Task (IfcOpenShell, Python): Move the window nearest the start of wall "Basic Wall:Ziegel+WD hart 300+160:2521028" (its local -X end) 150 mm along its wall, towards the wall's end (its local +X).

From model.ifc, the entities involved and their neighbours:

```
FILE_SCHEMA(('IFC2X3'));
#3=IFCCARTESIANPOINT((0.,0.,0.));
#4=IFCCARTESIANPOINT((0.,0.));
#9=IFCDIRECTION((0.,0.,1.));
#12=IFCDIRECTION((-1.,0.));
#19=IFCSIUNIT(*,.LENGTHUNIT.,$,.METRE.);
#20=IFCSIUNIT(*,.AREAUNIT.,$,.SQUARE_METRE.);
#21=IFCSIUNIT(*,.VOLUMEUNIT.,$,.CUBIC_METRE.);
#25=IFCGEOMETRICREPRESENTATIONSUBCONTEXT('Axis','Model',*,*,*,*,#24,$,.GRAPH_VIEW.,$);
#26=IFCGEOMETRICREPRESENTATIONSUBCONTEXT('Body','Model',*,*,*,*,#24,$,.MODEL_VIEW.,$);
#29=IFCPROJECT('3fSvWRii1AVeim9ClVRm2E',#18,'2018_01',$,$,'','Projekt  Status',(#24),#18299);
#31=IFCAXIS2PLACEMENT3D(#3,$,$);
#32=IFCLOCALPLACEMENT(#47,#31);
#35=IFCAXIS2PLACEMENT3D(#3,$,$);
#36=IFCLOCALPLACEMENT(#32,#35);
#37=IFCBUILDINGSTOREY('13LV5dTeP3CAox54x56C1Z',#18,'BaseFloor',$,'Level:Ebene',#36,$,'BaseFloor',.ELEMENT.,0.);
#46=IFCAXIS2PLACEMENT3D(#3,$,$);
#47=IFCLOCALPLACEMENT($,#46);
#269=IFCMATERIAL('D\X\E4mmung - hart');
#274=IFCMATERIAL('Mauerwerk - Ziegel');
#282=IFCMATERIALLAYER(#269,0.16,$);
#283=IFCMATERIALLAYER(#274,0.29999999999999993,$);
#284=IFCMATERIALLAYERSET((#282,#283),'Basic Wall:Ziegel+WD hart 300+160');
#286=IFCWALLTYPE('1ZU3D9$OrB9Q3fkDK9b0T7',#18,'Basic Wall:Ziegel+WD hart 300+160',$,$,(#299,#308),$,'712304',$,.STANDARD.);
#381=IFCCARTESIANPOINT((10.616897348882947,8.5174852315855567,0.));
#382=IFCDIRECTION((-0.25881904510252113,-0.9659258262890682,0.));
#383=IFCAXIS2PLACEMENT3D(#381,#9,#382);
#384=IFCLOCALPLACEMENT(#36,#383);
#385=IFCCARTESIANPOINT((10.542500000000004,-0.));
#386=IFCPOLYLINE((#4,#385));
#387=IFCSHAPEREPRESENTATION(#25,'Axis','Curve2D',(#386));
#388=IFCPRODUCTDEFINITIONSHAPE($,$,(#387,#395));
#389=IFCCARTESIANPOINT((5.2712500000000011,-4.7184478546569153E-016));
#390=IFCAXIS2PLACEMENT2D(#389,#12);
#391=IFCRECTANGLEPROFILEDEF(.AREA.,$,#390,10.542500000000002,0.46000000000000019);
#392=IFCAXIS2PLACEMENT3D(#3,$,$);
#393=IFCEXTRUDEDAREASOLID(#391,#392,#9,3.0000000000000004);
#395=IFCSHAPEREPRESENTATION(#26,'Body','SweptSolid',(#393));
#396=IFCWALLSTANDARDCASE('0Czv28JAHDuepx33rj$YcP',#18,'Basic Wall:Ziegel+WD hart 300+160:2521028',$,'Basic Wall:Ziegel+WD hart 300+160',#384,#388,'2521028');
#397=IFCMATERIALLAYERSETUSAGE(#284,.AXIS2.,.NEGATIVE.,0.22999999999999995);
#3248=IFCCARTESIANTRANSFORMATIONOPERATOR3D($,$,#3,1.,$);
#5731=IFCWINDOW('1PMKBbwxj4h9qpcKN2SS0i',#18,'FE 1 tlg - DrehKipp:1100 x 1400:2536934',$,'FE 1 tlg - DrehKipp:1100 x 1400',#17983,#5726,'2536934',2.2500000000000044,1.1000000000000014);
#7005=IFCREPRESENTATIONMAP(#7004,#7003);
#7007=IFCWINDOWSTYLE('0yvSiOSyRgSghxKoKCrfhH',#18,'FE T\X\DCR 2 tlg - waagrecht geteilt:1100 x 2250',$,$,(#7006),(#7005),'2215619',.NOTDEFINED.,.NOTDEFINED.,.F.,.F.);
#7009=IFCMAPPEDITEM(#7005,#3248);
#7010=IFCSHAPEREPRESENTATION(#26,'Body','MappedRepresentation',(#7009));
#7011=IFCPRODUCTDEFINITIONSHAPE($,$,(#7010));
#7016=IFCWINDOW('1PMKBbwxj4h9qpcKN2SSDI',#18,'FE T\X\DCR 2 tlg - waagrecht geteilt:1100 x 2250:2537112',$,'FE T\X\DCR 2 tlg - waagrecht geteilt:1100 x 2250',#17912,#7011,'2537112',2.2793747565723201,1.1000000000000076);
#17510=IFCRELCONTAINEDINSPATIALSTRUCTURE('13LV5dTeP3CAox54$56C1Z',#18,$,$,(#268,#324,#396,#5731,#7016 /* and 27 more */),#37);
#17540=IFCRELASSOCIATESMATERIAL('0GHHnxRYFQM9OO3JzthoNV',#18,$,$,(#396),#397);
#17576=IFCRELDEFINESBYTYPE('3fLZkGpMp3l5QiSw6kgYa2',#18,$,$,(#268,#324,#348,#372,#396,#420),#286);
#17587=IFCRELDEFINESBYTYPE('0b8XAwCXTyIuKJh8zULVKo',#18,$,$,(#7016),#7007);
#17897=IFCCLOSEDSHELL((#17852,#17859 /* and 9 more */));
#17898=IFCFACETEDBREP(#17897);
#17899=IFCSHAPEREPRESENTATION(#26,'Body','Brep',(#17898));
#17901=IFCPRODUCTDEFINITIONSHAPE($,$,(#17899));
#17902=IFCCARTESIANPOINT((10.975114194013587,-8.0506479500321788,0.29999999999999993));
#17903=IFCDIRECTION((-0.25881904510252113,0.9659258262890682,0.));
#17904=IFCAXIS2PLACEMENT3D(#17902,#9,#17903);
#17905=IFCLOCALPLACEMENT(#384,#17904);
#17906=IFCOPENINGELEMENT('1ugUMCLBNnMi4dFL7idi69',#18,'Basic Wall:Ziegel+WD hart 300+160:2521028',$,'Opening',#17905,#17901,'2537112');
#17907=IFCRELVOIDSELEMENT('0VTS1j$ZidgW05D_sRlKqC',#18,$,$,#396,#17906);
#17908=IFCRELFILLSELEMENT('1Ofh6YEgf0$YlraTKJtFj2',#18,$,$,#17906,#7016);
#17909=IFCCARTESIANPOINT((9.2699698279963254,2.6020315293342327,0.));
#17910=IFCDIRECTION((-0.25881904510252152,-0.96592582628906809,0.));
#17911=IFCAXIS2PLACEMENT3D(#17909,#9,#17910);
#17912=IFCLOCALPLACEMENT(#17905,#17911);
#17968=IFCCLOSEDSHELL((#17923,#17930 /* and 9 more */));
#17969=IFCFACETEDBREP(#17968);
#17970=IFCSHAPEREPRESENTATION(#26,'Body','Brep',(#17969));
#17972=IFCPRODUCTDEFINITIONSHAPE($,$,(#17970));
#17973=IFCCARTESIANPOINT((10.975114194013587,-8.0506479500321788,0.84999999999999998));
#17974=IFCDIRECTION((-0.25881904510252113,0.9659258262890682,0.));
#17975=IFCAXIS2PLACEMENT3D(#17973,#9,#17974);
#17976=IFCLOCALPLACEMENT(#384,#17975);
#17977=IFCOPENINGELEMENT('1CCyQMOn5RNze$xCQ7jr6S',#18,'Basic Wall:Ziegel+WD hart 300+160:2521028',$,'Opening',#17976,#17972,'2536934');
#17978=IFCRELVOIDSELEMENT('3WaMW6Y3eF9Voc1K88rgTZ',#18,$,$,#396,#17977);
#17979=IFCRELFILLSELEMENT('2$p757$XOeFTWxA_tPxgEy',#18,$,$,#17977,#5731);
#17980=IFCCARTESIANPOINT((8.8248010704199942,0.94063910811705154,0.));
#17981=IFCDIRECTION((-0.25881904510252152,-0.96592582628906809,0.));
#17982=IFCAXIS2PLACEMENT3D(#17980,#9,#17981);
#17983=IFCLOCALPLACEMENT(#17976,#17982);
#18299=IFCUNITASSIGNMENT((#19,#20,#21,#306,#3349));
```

```python
import ifcopenshell
import ifcopenshell.api.geometry
import ifcopenshell.util.placement
import ifcopenshell.util.unit

model = ifcopenshell.open("model.ifc")
unit_scale = ifcopenshell.util.unit.calculate_unit_scale(model)

window = model.by_guid("1PMKBbwxj4h9qpcKN2SSDI")
opening = window.FillsVoids[0].RelatingOpeningElement
wall = opening.VoidsElements[0].RelatingBuildingElement

wall_matrix = ifcopenshell.util.placement.get_local_placement(wall.ObjectPlacement)
shift = wall_matrix[:3, 0] * 0.15 / unit_scale
before = ifcopenshell.util.placement.get_local_placement(window.ObjectPlacement)[:3, 3].copy()

# The window is placed relative to its opening, so it follows when the opening moves.
matrix = ifcopenshell.util.placement.get_local_placement(opening.ObjectPlacement)
matrix[:3, 3] += shift
ifcopenshell.api.geometry.edit_object_placement(
    model, product=opening, matrix=matrix, is_si=False, should_transform_children=True
)

after = ifcopenshell.util.placement.get_local_placement(window.ObjectPlacement)[:3, 3]
print("window moved by", (after - before).round(3) + 0.0)

model.write("model_updated.ifc")
```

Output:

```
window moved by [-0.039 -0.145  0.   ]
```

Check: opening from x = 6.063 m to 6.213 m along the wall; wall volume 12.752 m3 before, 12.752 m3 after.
